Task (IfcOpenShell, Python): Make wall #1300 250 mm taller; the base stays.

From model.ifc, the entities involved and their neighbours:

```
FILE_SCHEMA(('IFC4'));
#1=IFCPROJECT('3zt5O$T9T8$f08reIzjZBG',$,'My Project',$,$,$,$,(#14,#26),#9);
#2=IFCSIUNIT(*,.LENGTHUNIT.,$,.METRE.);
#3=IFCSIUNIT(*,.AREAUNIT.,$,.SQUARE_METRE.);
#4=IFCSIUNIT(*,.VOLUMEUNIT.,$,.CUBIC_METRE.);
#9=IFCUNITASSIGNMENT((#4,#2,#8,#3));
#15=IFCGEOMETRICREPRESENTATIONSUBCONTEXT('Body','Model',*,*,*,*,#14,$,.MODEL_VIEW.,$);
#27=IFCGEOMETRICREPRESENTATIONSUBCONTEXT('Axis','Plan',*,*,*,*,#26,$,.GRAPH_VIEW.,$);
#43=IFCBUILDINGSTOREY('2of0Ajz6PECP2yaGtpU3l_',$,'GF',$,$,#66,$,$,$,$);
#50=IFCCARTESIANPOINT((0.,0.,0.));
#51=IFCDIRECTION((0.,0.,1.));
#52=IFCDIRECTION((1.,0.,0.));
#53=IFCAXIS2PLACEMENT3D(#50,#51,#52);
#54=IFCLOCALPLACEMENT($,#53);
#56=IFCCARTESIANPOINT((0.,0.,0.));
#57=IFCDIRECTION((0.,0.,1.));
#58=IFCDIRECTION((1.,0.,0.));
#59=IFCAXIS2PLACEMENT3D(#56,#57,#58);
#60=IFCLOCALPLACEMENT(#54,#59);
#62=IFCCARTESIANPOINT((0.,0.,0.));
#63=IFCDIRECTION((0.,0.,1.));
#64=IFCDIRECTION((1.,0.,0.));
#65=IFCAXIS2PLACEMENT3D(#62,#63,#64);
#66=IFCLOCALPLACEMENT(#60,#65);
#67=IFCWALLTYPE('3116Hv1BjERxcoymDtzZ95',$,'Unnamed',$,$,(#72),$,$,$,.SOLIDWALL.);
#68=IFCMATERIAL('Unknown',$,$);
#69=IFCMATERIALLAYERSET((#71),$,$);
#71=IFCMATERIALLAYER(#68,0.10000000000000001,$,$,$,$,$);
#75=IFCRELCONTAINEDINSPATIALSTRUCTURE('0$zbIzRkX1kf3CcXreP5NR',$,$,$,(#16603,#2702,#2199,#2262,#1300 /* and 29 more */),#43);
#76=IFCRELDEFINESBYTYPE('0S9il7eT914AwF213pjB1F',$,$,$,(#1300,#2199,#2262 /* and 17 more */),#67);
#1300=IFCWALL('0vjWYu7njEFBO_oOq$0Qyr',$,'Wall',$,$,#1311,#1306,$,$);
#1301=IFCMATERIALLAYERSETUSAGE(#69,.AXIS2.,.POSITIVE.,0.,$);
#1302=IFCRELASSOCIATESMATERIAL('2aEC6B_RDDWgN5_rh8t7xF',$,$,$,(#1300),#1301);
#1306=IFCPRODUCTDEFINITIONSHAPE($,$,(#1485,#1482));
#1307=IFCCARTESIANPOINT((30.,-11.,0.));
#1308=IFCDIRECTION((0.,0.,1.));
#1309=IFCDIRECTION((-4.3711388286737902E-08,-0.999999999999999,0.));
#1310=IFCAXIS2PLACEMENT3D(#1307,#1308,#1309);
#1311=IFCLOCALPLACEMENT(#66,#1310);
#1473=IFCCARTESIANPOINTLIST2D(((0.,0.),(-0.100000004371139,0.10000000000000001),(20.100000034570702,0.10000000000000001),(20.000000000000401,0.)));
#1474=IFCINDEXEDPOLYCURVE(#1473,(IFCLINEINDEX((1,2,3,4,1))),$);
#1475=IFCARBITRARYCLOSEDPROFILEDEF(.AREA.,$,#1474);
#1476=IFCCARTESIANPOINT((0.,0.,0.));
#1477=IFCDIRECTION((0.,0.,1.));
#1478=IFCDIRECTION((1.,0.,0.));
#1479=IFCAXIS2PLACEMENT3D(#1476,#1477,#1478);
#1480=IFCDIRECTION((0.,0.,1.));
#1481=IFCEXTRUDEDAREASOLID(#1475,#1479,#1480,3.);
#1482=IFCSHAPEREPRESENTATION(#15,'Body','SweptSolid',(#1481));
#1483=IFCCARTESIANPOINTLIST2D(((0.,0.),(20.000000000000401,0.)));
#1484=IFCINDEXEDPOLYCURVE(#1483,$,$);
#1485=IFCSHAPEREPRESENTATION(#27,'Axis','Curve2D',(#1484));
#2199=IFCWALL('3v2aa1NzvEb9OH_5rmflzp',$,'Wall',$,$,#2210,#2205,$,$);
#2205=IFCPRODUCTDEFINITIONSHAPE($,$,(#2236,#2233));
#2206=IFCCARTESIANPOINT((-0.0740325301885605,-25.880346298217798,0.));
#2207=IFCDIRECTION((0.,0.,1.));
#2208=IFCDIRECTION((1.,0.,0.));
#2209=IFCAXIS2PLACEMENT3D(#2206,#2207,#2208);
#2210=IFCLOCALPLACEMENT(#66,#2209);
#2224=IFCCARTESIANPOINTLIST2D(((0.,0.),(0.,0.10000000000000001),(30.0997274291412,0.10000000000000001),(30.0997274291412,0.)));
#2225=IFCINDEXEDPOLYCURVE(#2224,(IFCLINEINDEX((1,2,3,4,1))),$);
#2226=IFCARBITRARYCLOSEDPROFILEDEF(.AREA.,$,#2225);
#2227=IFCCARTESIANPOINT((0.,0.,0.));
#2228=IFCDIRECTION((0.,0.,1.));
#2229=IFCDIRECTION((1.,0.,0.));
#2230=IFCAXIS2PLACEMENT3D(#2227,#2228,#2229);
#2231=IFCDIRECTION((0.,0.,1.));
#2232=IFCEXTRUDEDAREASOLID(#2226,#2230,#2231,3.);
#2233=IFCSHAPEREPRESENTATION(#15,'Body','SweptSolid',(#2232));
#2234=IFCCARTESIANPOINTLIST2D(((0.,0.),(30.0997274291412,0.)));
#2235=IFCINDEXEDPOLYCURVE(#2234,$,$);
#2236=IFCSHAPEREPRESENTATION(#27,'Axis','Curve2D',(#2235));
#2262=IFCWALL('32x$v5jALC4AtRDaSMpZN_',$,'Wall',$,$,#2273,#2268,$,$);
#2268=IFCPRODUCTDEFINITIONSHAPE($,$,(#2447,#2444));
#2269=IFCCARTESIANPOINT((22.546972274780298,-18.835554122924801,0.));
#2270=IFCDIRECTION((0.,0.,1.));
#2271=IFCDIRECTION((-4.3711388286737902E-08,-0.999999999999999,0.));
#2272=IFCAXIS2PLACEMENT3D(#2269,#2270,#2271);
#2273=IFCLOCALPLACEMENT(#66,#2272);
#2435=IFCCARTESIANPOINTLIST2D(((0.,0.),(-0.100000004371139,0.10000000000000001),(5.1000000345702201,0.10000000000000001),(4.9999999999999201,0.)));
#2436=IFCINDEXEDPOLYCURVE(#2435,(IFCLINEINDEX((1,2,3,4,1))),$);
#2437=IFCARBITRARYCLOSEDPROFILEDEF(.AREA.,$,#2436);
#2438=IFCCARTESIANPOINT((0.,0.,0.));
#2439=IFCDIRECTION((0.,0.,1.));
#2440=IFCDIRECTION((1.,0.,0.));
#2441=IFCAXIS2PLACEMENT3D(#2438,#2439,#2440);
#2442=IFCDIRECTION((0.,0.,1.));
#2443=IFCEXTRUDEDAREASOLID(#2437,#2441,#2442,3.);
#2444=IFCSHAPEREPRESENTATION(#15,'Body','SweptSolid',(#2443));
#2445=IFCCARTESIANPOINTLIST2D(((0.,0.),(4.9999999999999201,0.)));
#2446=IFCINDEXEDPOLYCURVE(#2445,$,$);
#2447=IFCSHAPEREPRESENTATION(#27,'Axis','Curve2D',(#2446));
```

```python
import ifcopenshell
import ifcopenshell.geom
import ifcopenshell.util.representation
import ifcopenshell.util.shape
import ifcopenshell.util.unit

model = ifcopenshell.open("model.ifc")
unit_scale = ifcopenshell.util.unit.calculate_unit_scale(model)
settings = ifcopenshell.geom.settings()


def volume(element):
    """Net volume in cubic metres, openings subtracted."""
    shape = ifcopenshell.geom.create_shape(settings, element)
    return ifcopenshell.util.shape.get_volume(shape.geometry)


wall = model.by_guid("0vjWYu7njEFBO_oOq$0Qyr")
before = volume(wall)

body = ifcopenshell.util.representation.get_representation(wall, "Model", "Body")
solid = body.Items[0]
old_height = solid.Depth
solid.Depth += 0.25 / unit_scale
after = volume(wall)

print(f"height {old_height:g} -> {solid.Depth:g}, volume {before:.3f} -> {after:.3f} m3")

model.write("model_v2.ifc")
```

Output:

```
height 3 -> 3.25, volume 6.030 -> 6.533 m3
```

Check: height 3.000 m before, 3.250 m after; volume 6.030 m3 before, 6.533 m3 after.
